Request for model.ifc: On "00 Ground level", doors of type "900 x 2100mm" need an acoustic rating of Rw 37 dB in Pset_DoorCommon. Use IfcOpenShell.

First a look at what the model holds.

```python
import ifcopenshell
import ifcopenshell.util.element

model = ifcopenshell.open("model.ifc")
print(model.schema)
storey = next(s for s in model.by_type("IfcBuildingStorey") if s.Name == "00 Ground level")
doors = [e for e in ifcopenshell.util.element.get_decomposition(storey) if e.is_a("IfcDoor")]
seen = {}
for e in doors:
    element_type = ifcopenshell.util.element.get_type(e)
    key = (element_type.Name if element_type != e and element_type else None, ifcopenshell.util.element.get_pset(e, "Pset_DoorCommon", "AcousticRating"))
    seen[key] = seen.get(key, 0) + 1
for (name, value), count in sorted(seen.items(), key=str):
    print(count, "x", name, "|", value)
```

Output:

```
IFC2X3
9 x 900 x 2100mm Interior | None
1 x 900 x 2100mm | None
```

```python
import ifcopenshell
import ifcopenshell.api.pset
import ifcopenshell.util.element

model = ifcopenshell.open("model.ifc")

storey = next(s for s in model.by_type("IfcBuildingStorey") if s.Name == "00 Ground level")
doors = [e for e in ifcopenshell.util.element.get_decomposition(storey) if e.is_a("IfcDoor")]

count = 0
for e in doors:
    element_type = ifcopenshell.util.element.get_type(e)
    if element_type in (None, e) or element_type.Name != "900 x 2100mm":
        continue
    # add_pset returns the element's existing set when there is one.
    pset = ifcopenshell.api.pset.add_pset(model, product=e, name="Pset_DoorCommon")
    ifcopenshell.api.pset.edit_pset(model, pset=pset, properties={"AcousticRating": "Rw 37 dB"})
    count += 1

print(count, "doors updated")

model.write("model_rev.ifc")
```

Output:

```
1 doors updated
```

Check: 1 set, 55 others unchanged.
